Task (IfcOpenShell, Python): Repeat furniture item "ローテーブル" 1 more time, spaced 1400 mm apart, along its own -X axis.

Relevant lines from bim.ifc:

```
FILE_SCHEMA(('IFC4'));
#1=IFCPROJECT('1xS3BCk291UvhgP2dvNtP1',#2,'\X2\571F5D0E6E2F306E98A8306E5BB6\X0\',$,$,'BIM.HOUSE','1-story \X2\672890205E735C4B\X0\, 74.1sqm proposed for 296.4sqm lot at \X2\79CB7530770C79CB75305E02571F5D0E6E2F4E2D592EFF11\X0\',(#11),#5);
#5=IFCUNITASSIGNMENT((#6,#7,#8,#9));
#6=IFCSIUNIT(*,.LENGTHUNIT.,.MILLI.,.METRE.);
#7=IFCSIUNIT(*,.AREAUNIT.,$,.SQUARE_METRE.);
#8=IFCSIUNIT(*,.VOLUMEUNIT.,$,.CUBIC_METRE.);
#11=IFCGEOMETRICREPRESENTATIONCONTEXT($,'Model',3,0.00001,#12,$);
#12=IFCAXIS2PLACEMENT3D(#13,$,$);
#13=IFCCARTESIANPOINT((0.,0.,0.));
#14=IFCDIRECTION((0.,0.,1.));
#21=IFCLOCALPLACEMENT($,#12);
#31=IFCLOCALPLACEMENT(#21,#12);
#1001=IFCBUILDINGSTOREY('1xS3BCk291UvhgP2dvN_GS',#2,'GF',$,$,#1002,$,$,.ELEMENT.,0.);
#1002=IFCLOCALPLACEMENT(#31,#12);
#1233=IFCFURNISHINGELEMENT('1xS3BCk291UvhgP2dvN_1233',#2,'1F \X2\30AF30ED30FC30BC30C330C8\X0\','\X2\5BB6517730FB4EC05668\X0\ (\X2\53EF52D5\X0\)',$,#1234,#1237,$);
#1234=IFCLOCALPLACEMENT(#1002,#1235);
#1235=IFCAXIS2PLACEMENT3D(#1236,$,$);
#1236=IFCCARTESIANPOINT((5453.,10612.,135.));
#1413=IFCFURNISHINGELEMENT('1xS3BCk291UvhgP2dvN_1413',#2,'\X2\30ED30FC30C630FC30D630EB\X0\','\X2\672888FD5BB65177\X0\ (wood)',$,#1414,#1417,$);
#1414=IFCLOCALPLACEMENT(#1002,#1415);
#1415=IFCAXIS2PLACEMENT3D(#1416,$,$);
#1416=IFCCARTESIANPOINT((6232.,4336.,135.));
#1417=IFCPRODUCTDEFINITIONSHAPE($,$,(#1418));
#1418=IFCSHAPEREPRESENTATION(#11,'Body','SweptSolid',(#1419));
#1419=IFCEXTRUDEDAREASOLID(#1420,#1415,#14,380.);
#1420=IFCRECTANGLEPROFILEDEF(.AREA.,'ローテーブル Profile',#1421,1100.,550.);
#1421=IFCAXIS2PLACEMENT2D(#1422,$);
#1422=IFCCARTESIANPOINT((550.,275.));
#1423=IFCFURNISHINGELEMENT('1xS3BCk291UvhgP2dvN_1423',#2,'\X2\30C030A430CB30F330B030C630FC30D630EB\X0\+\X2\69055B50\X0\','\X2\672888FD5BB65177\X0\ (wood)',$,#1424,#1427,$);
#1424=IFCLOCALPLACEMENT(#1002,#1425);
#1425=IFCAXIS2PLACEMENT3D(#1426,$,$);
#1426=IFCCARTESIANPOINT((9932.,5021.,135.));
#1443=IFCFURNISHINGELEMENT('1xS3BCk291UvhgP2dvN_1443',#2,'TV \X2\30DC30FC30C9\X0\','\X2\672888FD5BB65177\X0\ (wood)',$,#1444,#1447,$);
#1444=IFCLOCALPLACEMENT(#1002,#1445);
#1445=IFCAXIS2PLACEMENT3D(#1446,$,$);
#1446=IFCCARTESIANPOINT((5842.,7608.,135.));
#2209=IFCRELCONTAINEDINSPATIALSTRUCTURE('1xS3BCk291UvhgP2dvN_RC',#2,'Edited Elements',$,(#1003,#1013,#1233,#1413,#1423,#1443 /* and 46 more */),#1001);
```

```python
import ifcopenshell
import ifcopenshell.api.geometry
import ifcopenshell.api.root
import ifcopenshell.util.element
import ifcopenshell.util.placement
import ifcopenshell.util.unit

model = ifcopenshell.open("bim.ifc")
unit_scale = ifcopenshell.util.unit.calculate_unit_scale(model)


def reuse_history(source, copy):
    """copy_class also copies each property set's owner history, people and application; keep the originals."""
    for rel in copy.IsDefinedBy:
        if rel.is_a("IfcRelDefinesByProperties") and (history := rel.RelatingPropertyDefinition.OwnerHistory):
            rel.RelatingPropertyDefinition.OwnerHistory = source.OwnerHistory
            ifcopenshell.util.element.remove_deep2(model, history)


source = model.by_guid("1xS3BCk291UvhgP2dvN_1413")
base = ifcopenshell.util.placement.get_local_placement(source.ObjectPlacement)
step = -base[:3, 0] * 1.4 / unit_scale

for i in range(1, 2):
    copy = ifcopenshell.api.root.copy_class(model, product=source)
    copy.Representation = ifcopenshell.util.element.copy_deep(
        model, source.Representation, exclude=["IfcGeometricRepresentationContext", "IfcRepresentationMap"]
    )
    reuse_history(source, copy)
    matrix = base.copy()
    matrix[:3, 3] += i * step
    print("added at", matrix[:3, 3].round(3) + 0.0)
    ifcopenshell.api.geometry.edit_object_placement(model, product=copy, matrix=matrix, is_si=False)

model.write("bim-out.ifc")
```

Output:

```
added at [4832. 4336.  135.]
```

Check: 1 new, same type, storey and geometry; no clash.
